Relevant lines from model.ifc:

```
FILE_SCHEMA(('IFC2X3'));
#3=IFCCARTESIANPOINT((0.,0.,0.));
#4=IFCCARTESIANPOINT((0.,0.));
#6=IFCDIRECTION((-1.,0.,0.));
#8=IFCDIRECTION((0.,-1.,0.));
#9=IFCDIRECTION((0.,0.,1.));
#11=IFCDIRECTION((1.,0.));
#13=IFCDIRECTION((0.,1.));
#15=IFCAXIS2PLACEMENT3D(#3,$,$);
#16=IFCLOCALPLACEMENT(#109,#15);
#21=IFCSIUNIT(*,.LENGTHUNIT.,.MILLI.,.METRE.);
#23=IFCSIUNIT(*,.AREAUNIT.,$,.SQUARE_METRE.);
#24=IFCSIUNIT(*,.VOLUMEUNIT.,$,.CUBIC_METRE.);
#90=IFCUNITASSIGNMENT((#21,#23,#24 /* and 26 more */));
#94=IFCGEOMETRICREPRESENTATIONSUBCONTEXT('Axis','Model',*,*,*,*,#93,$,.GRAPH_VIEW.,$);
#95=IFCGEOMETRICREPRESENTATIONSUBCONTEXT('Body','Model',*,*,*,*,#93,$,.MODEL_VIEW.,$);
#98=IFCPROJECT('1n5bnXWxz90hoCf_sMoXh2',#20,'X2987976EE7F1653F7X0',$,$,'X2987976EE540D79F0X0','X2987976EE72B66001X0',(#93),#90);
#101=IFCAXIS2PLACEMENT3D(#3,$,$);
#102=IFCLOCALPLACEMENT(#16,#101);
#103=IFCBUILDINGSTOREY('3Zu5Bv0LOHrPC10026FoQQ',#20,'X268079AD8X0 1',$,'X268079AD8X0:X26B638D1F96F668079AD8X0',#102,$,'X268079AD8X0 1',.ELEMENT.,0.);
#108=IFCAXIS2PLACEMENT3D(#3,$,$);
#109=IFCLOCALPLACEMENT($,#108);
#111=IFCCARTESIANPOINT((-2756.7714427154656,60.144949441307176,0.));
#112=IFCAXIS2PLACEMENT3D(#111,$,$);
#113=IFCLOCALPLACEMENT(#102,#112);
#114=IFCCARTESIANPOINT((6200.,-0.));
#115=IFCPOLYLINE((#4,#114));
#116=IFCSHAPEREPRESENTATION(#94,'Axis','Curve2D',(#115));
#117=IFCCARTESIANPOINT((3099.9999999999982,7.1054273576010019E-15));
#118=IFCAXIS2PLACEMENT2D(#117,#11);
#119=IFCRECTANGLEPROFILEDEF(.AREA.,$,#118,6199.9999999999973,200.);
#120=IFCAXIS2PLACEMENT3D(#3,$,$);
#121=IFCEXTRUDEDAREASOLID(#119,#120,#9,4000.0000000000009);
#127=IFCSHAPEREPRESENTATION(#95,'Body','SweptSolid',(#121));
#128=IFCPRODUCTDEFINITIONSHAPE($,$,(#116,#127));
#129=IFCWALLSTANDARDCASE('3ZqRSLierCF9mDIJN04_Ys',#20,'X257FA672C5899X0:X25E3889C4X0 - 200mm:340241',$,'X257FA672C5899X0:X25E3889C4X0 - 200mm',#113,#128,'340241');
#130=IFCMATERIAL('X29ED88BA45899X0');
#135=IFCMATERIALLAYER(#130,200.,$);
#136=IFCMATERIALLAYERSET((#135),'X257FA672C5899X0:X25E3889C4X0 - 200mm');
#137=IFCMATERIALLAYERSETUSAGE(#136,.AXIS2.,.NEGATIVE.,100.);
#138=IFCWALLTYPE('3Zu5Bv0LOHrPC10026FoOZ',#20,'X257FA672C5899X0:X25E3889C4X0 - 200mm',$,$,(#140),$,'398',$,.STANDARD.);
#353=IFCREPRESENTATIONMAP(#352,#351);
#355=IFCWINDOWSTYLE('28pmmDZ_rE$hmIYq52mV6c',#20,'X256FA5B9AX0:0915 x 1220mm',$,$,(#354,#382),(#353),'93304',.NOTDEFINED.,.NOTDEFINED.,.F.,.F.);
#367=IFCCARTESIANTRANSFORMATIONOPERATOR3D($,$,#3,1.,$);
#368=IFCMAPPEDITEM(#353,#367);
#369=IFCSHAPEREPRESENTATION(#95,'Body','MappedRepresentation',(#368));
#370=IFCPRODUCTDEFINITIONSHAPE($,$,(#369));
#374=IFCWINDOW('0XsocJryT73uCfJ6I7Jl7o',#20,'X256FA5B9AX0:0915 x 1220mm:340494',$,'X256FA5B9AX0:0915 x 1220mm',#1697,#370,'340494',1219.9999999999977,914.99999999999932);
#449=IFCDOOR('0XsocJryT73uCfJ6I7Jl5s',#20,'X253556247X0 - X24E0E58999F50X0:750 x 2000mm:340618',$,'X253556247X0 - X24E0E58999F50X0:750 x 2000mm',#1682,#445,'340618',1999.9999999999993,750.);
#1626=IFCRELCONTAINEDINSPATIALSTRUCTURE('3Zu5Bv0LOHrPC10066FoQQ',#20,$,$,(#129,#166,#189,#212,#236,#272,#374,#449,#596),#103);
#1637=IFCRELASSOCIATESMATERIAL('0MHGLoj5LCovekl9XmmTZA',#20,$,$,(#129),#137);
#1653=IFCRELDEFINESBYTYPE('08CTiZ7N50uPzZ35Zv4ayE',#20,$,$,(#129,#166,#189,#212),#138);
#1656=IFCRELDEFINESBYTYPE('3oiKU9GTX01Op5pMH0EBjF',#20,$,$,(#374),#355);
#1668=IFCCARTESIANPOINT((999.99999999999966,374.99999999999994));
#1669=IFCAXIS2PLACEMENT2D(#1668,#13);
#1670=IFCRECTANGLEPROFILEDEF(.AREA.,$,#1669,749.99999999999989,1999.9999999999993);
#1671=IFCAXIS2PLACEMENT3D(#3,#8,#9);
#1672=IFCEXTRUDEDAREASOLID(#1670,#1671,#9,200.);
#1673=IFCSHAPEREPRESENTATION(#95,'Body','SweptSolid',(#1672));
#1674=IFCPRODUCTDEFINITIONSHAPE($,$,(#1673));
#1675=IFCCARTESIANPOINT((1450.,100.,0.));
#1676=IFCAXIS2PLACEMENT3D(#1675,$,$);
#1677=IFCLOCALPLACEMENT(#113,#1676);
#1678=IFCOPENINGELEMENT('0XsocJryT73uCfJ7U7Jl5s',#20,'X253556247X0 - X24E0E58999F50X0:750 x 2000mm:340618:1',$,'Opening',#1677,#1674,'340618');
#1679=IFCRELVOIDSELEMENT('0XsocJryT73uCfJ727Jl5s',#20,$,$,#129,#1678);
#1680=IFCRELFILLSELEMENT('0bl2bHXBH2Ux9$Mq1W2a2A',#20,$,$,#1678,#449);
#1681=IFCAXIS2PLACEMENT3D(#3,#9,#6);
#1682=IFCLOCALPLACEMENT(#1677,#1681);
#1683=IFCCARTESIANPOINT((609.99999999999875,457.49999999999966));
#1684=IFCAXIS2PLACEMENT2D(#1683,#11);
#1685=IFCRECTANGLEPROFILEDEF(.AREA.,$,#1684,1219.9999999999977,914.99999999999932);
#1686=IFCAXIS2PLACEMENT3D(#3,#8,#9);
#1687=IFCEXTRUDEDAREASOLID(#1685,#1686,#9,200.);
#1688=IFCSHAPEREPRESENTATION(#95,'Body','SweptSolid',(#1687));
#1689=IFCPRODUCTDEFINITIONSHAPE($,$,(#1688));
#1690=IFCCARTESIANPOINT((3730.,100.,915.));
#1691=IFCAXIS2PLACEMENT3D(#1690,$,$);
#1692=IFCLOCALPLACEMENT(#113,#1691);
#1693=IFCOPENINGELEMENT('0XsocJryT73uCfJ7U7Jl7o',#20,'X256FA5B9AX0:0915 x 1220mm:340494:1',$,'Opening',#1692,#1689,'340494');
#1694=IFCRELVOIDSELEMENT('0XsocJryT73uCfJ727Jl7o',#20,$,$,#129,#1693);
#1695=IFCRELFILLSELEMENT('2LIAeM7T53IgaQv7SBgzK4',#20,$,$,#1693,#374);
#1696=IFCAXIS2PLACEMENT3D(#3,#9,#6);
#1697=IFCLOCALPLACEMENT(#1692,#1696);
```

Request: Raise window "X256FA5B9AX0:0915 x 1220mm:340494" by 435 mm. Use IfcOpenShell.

```python
import numpy as np
import ifcopenshell
import ifcopenshell.api.geometry
import ifcopenshell.util.placement
import ifcopenshell.util.unit

model = ifcopenshell.open("model.ifc")
unit_scale = ifcopenshell.util.unit.calculate_unit_scale(model)

window = model.by_id(374)
opening = window.FillsVoids[0].RelatingOpeningElement
dz = 0.435 / unit_scale

shift = np.array([0.0, 0.0, dz])
# The window is placed relative to its opening, so it follows when the opening moves.
matrix = ifcopenshell.util.placement.get_local_placement(opening.ObjectPlacement)
matrix[:3, 3] += shift
ifcopenshell.api.geometry.edit_object_placement(
    model, product=opening, matrix=matrix, is_si=False, should_transform_children=True
)

print(f"moved by {dz * unit_scale:+.3f} m")

model.write("model_rev.ifc")
```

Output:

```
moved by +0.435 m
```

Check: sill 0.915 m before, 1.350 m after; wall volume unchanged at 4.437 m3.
